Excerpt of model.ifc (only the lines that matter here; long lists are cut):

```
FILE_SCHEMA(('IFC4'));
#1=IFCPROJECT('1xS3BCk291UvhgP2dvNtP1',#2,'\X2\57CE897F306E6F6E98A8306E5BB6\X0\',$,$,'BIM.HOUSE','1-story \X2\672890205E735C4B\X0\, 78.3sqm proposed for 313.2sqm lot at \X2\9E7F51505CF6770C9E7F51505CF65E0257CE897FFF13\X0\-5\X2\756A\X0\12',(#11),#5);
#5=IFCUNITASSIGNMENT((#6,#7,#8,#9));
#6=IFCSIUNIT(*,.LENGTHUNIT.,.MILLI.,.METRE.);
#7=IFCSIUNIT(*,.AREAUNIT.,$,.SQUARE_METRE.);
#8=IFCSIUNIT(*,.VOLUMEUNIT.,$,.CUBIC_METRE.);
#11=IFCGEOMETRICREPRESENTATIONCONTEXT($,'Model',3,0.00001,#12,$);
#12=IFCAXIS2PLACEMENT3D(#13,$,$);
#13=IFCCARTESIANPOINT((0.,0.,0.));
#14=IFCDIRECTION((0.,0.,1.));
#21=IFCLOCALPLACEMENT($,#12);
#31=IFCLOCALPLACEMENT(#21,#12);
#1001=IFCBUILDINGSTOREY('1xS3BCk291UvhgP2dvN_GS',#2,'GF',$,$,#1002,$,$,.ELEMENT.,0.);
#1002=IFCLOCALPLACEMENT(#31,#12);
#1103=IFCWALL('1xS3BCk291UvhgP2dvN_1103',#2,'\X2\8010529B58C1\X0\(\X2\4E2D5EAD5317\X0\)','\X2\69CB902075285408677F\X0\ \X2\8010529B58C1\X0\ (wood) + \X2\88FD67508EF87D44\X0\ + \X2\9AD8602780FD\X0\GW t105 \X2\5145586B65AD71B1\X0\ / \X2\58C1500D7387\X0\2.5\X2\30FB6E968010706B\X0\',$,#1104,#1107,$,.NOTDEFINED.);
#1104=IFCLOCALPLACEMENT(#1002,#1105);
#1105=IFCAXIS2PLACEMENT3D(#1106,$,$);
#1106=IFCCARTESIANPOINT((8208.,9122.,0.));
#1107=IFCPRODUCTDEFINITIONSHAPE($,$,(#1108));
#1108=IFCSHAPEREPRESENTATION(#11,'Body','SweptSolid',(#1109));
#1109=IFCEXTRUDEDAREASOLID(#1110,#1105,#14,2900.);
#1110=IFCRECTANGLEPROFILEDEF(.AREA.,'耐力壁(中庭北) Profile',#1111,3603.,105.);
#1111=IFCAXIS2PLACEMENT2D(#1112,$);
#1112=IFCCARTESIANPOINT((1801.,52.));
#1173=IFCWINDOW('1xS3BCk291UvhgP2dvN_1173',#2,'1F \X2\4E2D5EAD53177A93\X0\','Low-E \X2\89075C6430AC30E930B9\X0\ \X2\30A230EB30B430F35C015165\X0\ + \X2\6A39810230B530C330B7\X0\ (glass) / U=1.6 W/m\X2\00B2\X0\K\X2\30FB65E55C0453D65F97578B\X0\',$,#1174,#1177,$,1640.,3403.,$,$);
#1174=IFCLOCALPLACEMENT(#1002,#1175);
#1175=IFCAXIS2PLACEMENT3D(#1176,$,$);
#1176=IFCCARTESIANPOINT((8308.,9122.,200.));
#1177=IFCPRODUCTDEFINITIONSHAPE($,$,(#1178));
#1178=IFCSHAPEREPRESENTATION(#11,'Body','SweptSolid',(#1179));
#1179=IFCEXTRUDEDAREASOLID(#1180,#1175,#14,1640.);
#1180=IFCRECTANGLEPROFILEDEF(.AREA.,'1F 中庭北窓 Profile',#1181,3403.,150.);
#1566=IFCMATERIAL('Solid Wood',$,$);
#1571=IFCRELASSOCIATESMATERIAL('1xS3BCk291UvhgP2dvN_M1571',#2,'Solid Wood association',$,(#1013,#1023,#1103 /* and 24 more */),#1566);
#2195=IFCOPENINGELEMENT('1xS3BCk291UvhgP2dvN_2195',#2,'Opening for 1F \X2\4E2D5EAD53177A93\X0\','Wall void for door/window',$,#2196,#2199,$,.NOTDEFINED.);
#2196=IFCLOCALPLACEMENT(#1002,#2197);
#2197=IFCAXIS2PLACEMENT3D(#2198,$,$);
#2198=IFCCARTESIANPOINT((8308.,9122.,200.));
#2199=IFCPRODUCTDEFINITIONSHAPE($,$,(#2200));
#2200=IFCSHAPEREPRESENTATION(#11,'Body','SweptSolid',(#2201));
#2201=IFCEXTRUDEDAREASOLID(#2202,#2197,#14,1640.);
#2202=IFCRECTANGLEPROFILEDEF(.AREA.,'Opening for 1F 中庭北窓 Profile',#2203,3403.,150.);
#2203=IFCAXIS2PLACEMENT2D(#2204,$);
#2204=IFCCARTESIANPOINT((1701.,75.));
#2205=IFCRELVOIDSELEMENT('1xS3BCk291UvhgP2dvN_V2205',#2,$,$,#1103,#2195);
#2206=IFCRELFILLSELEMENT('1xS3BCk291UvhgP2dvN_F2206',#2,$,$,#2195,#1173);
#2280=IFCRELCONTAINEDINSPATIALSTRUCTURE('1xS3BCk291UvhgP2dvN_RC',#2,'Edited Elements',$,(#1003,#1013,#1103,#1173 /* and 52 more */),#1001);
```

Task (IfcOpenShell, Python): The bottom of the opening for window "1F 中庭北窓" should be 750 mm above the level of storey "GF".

```python
import numpy as np
import ifcopenshell
import ifcopenshell.api.geometry
import ifcopenshell.geom
import ifcopenshell.util.element
import ifcopenshell.util.placement
import ifcopenshell.util.shape
import ifcopenshell.util.unit

model = ifcopenshell.open("model.ifc")
unit_scale = ifcopenshell.util.unit.calculate_unit_scale(model)

window = model.by_guid("1xS3BCk291UvhgP2dvN_1173")
opening = window.FillsVoids[0].RelatingOpeningElement
storey = ifcopenshell.util.element.get_container(window, ifc_class="IfcBuildingStorey")
level = ifcopenshell.util.placement.get_local_placement(storey.ObjectPlacement)[2, 3]

# The opening's origin need not be at the sill, so measure its lowest point.
shape = ifcopenshell.geom.create_shape(ifcopenshell.geom.settings(), opening)
bottom = ifcopenshell.util.shape.get_shape_bottom_elevation(shape, shape.geometry) / unit_scale
dz = level + 0.75 / unit_scale - bottom

shift = np.array([0.0, 0.0, dz])
# The window is not placed relative to its opening, so move both.
for product in (opening, window):
    matrix = ifcopenshell.util.placement.get_local_placement(product.ObjectPlacement)
    matrix[:3, 3] += shift
    ifcopenshell.api.geometry.edit_object_placement(model, product=product, matrix=matrix, is_si=False)

print(f"moved by {dz * unit_scale:+.3f} m")

model.write("model_v2.ifc")
```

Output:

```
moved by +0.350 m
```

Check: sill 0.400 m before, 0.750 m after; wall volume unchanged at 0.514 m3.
